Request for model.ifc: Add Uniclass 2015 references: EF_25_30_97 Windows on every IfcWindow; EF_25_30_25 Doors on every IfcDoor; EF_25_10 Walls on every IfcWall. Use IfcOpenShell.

First a look at what the model holds.

```python
import ifcopenshell

model = ifcopenshell.open("model.ifc")
print(model.schema)
print("classifications:", [c.Name for c in model.by_type("IfcClassification")])
for ifc_class in ("IfcDoor", "IfcRoof", "IfcStair", "IfcWall", "IfcWindow"):
    print(ifc_class, len(model.by_type(ifc_class)))
```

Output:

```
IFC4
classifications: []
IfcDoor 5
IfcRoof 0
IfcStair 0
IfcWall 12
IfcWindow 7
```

```python
import ifcopenshell
import ifcopenshell.api.classification

model = ifcopenshell.open("model.ifc")

system = ifcopenshell.api.classification.add_classification(model, classification="Uniclass 2015")

codes = {
    "IfcWindow": ("EF_25_30_97", "Windows"),
    "IfcDoor": ("EF_25_30_25", "Doors"),
    "IfcWall": ("EF_25_10", "Walls"),
}
for ifc_class, (code, name) in codes.items():
    products = model.by_type(ifc_class)
    ifcopenshell.api.classification.add_reference(
        model, products=products, classification=system, identification=code, name=name
    )
    print(code, len(products))

model.write("model_updated.ifc")
```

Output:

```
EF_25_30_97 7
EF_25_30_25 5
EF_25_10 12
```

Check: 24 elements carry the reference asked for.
